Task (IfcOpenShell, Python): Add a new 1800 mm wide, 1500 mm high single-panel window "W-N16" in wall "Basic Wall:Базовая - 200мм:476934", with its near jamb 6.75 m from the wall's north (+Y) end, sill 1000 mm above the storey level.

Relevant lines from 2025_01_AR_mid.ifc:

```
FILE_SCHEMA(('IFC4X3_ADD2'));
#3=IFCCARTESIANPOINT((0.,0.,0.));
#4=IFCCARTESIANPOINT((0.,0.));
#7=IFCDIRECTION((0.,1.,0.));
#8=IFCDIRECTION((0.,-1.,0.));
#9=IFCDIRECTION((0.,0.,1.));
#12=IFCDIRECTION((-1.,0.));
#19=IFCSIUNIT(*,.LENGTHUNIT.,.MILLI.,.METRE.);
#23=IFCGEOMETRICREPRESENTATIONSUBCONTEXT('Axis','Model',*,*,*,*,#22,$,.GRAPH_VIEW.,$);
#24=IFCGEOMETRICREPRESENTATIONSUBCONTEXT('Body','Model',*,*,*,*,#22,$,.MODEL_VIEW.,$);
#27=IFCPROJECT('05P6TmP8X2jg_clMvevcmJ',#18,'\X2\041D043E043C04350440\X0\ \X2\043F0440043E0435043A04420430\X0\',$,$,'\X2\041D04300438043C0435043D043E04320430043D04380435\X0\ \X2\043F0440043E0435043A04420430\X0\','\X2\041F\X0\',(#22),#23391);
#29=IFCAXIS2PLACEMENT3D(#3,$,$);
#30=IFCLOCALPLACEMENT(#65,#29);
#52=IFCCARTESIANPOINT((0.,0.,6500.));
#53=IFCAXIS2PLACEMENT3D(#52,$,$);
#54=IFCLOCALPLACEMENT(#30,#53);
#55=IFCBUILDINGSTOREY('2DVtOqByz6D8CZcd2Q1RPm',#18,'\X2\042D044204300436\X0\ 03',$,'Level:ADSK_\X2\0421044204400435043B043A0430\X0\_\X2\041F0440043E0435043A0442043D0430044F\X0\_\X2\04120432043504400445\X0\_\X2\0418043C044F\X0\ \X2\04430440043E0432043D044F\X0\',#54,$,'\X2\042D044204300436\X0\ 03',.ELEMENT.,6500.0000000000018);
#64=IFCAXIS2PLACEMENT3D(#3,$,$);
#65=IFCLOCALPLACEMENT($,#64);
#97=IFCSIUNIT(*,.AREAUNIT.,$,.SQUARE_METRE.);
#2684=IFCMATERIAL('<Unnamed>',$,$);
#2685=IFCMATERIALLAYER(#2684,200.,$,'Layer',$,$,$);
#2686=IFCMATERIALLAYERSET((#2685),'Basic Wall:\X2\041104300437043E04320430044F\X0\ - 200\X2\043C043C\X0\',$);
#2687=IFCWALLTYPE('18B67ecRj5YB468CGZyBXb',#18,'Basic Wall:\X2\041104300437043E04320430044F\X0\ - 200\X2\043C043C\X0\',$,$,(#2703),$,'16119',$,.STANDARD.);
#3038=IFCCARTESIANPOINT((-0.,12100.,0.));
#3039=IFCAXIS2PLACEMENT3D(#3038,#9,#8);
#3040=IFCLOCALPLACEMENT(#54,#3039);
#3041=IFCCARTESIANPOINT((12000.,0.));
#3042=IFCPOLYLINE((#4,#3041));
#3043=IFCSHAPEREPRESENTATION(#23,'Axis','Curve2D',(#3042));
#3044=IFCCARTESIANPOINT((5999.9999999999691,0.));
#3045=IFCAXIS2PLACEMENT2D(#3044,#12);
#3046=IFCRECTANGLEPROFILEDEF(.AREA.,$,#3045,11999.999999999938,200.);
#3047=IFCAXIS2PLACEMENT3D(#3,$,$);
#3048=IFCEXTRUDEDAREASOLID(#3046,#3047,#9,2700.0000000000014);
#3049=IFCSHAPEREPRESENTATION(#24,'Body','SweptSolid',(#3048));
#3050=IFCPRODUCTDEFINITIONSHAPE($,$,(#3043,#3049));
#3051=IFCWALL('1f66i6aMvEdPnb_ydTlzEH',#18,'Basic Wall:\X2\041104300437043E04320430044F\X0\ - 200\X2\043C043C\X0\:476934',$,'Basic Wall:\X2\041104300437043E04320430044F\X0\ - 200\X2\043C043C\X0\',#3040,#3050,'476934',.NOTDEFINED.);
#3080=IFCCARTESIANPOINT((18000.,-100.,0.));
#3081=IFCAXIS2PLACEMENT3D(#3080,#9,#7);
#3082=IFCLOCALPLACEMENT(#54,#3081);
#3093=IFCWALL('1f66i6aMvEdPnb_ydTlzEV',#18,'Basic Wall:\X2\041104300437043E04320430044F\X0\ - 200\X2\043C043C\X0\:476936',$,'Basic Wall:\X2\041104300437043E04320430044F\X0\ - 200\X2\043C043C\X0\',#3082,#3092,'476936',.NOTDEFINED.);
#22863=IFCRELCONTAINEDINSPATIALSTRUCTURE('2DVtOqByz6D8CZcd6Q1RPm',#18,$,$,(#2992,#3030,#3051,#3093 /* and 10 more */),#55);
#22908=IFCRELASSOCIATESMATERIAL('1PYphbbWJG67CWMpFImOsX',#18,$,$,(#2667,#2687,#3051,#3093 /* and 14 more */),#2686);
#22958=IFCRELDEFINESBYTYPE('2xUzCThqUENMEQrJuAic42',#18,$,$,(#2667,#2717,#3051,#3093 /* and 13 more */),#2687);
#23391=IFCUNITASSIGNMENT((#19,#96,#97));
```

```python
import numpy as np
import ifcopenshell
import ifcopenshell.api.feature
import ifcopenshell.api.geometry
import ifcopenshell.api.root
import ifcopenshell.api.spatial
import ifcopenshell.geom
import ifcopenshell.util.element
import ifcopenshell.util.placement
import ifcopenshell.util.representation
import ifcopenshell.util.shape
import ifcopenshell.util.unit

model = ifcopenshell.open("2025_01_AR_mid.ifc")
unit_scale = ifcopenshell.util.unit.calculate_unit_scale(model)
settings = ifcopenshell.geom.settings()


def volume(element):
    """Net volume in cubic metres, openings subtracted."""
    shape = ifcopenshell.geom.create_shape(settings, element)
    return ifcopenshell.util.shape.get_volume(shape.geometry)


wall = model.by_id(3051)
storey = ifcopenshell.util.element.get_container(wall, ifc_class="IfcBuildingStorey")
context = ifcopenshell.util.representation.get_context(model, "Model", "Body", "MODEL_VIEW")
before = volume(wall)

width, height, from_end, sill = 1.8, 1.5, 6.75, 1  # metres

# The wall runs along its own X axis, and the end named is its -X end.
wall_shape = ifcopenshell.geom.create_shape(settings, wall)
x, y, z = ifcopenshell.util.shape.get_vertices(wall_shape.geometry).T
start = x.min() + from_end
face, thickness = float(y.min()), float(y.max() - y.min())
wall_matrix = ifcopenshell.util.placement.get_local_placement(wall.ObjectPlacement)
level = ifcopenshell.util.placement.get_local_placement(storey.ObjectPlacement)[2, 3]


def in_wall(x, y):
    """Placement at x, y metres in the wall's axes, at sill height."""
    matrix = wall_matrix.copy()
    matrix[:, 3] = wall_matrix @ np.array([x / unit_scale, y / unit_scale, 0.0, 1.0])
    matrix[2, 3] = level + sill / unit_scale
    return matrix


# Opening: a box that overshoots both wall faces by 50 mm.
opening = ifcopenshell.api.root.create_entity(model, ifc_class="IfcOpeningElement", predefined_type="OPENING")
box = ifcopenshell.api.geometry.add_wall_representation(
    model, context=context, length=width, height=height, thickness=thickness + 0.1
)
ifcopenshell.api.geometry.assign_representation(model, product=opening, representation=box)
ifcopenshell.api.geometry.edit_object_placement(model, product=opening, matrix=in_wall(start, face - 0.05), is_si=False)
ifcopenshell.api.feature.add_feature(model, feature=opening, element=wall)

window = ifcopenshell.api.root.create_entity(model, ifc_class="IfcWindow", name="W-N16", predefined_type="WINDOW")
window.OverallWidth, window.OverallHeight = width / unit_scale, height / unit_scale
window.PartitioningType = "SINGLE_PANEL"
body = ifcopenshell.api.geometry.add_window_representation(
    model,
    context=context,
    overall_width=window.OverallWidth,
    overall_height=window.OverallHeight,
    partition_type="SINGLE_PANEL",
)
ifcopenshell.api.geometry.assign_representation(model, product=window, representation=body)
ifcopenshell.api.spatial.assign_container(model, products=[window], relating_structure=storey)
ifcopenshell.api.feature.add_filling(model, opening=opening, element=window)

# Centre the window in the wall's thickness.
ifcopenshell.api.geometry.edit_object_placement(model, product=window, matrix=in_wall(start, face), is_si=False)
window_shape = ifcopenshell.geom.create_shape(settings, window)
depth = ifcopenshell.util.shape.get_vertices(window_shape.geometry)[:, 1]
offset = face + thickness / 2 - (depth.min() + depth.max()) / 2
ifcopenshell.api.geometry.edit_object_placement(model, product=window, matrix=in_wall(start, offset), is_si=False)

after = volume(wall)

print(f"wall volume {before:.3f} -> {after:.3f} m3")

model.write("2025_01_AR_mid_edited.ifc")
```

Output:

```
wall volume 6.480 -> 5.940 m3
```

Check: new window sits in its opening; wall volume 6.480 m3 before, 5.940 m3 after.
